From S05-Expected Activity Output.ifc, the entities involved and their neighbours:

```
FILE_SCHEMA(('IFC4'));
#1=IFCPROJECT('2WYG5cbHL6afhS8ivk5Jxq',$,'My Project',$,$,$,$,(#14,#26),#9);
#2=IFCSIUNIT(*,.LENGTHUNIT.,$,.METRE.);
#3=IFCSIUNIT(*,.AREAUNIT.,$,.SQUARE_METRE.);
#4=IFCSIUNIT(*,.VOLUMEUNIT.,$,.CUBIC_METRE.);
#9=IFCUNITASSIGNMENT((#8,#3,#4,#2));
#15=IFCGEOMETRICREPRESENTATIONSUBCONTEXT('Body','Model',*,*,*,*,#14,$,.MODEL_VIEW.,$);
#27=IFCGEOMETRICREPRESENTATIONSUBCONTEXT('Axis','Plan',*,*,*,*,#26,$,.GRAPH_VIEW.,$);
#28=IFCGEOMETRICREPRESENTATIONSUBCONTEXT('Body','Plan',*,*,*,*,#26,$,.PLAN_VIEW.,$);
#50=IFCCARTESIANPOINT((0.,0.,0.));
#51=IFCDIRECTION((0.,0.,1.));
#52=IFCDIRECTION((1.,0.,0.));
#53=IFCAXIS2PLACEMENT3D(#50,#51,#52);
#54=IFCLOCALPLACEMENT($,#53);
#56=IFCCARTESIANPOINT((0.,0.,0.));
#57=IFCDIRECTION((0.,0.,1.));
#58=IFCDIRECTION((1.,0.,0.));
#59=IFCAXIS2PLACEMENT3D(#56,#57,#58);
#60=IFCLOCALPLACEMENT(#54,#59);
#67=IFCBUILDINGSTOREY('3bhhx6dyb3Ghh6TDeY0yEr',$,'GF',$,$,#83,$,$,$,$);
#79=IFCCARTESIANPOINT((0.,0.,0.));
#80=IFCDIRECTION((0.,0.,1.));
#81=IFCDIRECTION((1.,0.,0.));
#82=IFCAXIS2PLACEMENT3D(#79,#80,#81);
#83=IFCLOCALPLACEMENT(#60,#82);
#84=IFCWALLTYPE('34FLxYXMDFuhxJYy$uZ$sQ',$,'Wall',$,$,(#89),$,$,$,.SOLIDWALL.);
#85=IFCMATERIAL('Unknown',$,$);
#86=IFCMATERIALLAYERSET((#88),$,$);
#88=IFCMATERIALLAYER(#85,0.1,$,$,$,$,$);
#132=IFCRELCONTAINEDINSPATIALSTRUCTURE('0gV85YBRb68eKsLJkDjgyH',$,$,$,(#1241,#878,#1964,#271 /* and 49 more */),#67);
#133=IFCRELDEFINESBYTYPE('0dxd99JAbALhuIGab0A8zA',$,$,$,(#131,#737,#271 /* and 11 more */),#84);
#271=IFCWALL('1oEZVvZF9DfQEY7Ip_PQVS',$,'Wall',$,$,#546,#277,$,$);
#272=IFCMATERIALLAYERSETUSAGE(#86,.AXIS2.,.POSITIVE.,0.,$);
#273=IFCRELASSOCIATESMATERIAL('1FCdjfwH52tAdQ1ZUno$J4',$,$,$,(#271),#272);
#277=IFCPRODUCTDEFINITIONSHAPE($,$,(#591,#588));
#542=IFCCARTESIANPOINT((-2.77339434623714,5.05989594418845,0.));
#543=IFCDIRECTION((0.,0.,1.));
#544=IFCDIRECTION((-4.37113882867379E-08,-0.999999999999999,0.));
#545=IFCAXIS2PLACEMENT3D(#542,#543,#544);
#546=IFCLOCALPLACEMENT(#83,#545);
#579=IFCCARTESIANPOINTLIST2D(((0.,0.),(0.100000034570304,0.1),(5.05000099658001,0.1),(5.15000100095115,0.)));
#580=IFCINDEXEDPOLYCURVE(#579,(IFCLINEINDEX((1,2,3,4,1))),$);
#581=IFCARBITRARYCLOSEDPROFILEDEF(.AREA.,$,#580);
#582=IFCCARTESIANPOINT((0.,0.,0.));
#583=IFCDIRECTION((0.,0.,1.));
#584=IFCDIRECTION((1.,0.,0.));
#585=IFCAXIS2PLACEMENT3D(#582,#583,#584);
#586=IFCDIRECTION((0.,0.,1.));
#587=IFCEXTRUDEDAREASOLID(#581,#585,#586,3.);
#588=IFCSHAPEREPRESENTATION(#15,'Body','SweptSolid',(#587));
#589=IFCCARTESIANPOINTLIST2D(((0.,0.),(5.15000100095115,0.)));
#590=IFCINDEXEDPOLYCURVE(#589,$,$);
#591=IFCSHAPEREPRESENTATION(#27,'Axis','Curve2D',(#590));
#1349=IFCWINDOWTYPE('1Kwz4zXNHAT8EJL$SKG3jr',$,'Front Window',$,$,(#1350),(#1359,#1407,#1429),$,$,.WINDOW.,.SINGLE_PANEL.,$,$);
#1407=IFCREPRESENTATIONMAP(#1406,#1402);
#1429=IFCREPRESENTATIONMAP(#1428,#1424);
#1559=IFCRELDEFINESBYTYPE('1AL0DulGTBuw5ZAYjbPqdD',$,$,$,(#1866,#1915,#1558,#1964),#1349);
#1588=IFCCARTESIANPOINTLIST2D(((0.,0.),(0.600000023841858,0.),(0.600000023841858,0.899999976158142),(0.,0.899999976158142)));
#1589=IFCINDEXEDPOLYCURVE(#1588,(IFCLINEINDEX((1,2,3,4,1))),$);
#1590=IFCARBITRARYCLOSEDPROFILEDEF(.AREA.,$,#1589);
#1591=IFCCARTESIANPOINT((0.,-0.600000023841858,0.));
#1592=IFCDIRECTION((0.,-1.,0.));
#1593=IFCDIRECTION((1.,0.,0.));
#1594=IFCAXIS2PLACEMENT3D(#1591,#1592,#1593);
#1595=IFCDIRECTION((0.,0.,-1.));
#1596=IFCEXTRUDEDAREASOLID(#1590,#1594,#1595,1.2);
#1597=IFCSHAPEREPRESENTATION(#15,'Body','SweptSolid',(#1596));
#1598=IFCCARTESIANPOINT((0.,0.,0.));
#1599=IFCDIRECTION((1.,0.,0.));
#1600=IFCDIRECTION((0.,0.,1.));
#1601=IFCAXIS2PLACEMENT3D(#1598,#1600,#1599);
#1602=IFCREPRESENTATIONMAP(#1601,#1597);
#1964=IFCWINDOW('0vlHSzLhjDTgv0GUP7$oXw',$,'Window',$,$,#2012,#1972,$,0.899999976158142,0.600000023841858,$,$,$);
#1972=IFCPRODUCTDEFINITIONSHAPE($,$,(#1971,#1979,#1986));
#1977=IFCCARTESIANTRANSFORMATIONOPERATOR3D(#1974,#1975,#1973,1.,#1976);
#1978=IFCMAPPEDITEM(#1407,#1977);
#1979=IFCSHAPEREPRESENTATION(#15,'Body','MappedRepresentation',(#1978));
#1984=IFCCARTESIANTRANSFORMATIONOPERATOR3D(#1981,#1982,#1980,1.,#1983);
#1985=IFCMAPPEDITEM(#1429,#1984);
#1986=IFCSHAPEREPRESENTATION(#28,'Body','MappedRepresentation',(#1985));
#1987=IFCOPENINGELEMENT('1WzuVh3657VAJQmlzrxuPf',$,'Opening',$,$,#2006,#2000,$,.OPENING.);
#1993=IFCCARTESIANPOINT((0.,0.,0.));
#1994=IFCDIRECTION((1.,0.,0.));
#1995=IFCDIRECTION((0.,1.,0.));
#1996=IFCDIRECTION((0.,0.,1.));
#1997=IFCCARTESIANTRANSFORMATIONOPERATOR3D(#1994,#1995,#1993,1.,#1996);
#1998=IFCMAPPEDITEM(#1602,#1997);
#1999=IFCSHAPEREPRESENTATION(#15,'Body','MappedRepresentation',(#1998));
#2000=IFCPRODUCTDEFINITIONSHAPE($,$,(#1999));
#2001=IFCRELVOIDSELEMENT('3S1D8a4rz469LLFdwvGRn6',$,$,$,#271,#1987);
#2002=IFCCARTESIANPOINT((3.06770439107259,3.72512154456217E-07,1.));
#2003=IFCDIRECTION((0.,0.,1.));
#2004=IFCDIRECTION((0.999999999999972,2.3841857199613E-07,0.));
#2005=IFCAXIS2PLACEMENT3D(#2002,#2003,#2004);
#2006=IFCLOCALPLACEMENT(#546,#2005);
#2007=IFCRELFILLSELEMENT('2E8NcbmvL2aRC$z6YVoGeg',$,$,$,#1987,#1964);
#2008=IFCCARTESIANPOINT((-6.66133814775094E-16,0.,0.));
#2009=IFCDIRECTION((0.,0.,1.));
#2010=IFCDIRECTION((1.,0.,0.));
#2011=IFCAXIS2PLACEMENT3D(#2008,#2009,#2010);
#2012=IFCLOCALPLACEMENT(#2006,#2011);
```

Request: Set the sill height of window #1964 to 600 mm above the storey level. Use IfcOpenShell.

```python
import numpy as np
import ifcopenshell
import ifcopenshell.api.geometry
import ifcopenshell.geom
import ifcopenshell.util.element
import ifcopenshell.util.placement
import ifcopenshell.util.shape
import ifcopenshell.util.unit

model = ifcopenshell.open("S05-Expected Activity Output.ifc")
unit_scale = ifcopenshell.util.unit.calculate_unit_scale(model)

window = model.by_guid("0vlHSzLhjDTgv0GUP7$oXw")
opening = window.FillsVoids[0].RelatingOpeningElement
storey = ifcopenshell.util.element.get_container(window, ifc_class="IfcBuildingStorey")
level = ifcopenshell.util.placement.get_local_placement(storey.ObjectPlacement)[2, 3]

# The opening's origin need not be at the sill, so measure its lowest point.
shape = ifcopenshell.geom.create_shape(ifcopenshell.geom.settings(), opening)
bottom = ifcopenshell.util.shape.get_shape_bottom_elevation(shape, shape.geometry) / unit_scale
dz = level + 0.6 / unit_scale - bottom

shift = np.array([0.0, 0.0, dz])
# The window is placed relative to its opening, so it follows when the opening moves.
matrix = ifcopenshell.util.placement.get_local_placement(opening.ObjectPlacement)
matrix[:3, 3] += shift
ifcopenshell.api.geometry.edit_object_placement(
    model, product=opening, matrix=matrix, is_si=False, should_transform_children=True
)

print(f"moved by {dz * unit_scale:+.3f} m")

model.write("S05-Expected Activity Output_updated.ifc")
```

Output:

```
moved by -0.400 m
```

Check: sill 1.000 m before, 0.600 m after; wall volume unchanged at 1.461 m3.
